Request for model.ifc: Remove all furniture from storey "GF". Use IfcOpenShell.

First a look at what the model holds.

```python
import ifcopenshell
import ifcopenshell.util.element

model = ifcopenshell.open("model.ifc")
print(model.schema)
storey = next(s for s in model.by_type("IfcBuildingStorey") if s.Name == "GF")
furniture = [e for e in ifcopenshell.util.element.get_decomposition(storey) if e.is_a("IfcFurnishingElement")]
seen = {}
for e in furniture:
    element_type = ifcopenshell.util.element.get_type(e)
    name = element_type.Name if element_type not in (None, e) else None
    seen[name] = seen.get(name, 0) + 1
for name, count in sorted(seen.items(), key=str):
    print(count, "x", name)
```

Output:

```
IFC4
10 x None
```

```python
import ifcopenshell
import ifcopenshell.api.root
import ifcopenshell.util.element

model = ifcopenshell.open("model.ifc")

storey = next(s for s in model.by_type("IfcBuildingStorey") if s.Name == "GF")
furniture = [e for e in ifcopenshell.util.element.get_decomposition(storey) if e.is_a("IfcFurnishingElement")]

for e in furniture:
    ifcopenshell.api.root.remove_product(model, product=e)
print(len(furniture), "removed")

model.write("model_updated.ifc")
```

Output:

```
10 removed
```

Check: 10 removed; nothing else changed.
